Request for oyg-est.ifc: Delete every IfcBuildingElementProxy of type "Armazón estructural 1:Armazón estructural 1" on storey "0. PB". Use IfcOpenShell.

First a look at what the model holds.

```python
import ifcopenshell
import ifcopenshell.util.element

model = ifcopenshell.open("oyg-est.ifc")
print(model.schema)
storey = next(s for s in model.by_type("IfcBuildingStorey") if s.Name == "0. PB")
proxies = [e for e in ifcopenshell.util.element.get_decomposition(storey) if e.is_a("IfcBuildingElementProxy")]
seen = {}
for e in proxies:
    element_type = ifcopenshell.util.element.get_type(e)
    name = element_type.Name if element_type not in (None, e) else None
    seen[name] = seen.get(name, 0) + 1
for name, count in sorted(seen.items(), key=str):
    print(count, "x", name)
```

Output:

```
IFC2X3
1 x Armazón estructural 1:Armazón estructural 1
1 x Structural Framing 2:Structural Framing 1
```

```python
import ifcopenshell
import ifcopenshell.api.root
import ifcopenshell.util.element

model = ifcopenshell.open("oyg-est.ifc")

storey = next(s for s in model.by_type("IfcBuildingStorey") if s.Name == "0. PB")
proxies = [e for e in ifcopenshell.util.element.get_decomposition(storey) if e.is_a("IfcBuildingElementProxy")]
targets = [e for e in proxies if (t := ifcopenshell.util.element.get_type(e)) not in (None, e) and t.Name == "Armazón estructural 1:Armazón estructural 1"]

for e in targets:
    ifcopenshell.api.root.remove_product(model, product=e)
print(len(targets), "removed")

model.write("oyg-est_rev.ifc")
```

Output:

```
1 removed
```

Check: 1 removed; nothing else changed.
